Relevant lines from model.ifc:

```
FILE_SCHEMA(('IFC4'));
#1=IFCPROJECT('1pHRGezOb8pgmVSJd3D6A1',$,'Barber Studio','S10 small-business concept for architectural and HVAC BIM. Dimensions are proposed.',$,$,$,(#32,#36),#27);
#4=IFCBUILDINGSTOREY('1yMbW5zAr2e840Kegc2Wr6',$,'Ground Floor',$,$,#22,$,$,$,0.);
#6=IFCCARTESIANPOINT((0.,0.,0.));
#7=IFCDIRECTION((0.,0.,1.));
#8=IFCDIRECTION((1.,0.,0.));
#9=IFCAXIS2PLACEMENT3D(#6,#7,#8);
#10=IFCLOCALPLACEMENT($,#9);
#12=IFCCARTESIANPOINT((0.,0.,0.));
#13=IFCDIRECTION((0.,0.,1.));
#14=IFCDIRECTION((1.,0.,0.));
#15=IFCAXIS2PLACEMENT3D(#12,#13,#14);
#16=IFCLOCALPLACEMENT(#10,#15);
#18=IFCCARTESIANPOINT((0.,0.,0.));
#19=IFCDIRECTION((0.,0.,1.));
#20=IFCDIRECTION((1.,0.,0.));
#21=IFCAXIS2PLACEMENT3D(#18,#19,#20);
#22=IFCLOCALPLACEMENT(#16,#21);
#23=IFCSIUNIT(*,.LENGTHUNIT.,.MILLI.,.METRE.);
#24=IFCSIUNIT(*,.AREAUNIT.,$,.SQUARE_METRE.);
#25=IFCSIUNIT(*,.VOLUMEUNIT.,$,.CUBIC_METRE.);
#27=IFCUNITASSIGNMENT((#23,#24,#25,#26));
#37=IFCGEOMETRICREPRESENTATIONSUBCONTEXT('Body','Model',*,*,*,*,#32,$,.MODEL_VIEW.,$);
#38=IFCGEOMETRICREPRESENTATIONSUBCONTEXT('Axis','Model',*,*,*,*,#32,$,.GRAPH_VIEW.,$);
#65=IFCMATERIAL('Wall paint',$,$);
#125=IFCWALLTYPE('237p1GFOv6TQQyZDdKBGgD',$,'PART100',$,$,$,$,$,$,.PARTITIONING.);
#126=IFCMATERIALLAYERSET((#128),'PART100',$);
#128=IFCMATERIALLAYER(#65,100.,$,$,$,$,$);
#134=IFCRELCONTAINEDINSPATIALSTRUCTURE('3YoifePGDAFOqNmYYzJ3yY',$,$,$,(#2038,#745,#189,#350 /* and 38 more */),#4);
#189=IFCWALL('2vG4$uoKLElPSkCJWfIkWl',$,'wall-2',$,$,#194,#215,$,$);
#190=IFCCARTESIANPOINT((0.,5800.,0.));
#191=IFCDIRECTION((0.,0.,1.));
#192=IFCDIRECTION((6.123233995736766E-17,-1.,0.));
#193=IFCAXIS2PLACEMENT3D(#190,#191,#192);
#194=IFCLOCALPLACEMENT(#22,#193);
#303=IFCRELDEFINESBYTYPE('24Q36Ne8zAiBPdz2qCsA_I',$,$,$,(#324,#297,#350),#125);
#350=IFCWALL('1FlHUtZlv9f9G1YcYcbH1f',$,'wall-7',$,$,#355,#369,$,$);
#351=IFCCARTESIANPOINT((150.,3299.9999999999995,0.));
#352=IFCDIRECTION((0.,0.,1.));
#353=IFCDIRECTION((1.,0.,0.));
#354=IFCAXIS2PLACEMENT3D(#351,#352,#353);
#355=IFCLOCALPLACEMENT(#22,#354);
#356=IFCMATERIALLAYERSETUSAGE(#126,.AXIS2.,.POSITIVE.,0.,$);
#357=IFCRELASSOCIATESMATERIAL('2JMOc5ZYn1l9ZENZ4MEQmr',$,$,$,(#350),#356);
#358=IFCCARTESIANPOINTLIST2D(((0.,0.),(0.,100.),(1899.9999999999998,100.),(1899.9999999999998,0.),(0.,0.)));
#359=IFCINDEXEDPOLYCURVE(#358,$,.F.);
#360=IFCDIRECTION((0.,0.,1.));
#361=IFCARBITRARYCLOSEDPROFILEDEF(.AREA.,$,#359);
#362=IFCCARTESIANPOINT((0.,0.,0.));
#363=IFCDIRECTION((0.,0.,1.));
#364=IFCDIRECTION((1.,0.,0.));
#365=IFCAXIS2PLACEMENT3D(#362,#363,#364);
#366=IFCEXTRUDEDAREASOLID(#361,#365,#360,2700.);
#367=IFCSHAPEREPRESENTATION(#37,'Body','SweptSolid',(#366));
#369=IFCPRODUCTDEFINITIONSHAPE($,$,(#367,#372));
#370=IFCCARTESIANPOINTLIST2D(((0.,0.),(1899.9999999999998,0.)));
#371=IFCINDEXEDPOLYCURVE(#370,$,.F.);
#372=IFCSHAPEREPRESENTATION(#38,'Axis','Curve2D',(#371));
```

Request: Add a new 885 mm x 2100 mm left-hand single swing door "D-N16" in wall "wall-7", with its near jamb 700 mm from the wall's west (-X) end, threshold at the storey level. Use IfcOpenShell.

```python
import numpy as np
import ifcopenshell
import ifcopenshell.api.feature
import ifcopenshell.api.geometry
import ifcopenshell.api.root
import ifcopenshell.api.spatial
import ifcopenshell.geom
import ifcopenshell.util.element
import ifcopenshell.util.placement
import ifcopenshell.util.representation
import ifcopenshell.util.shape
import ifcopenshell.util.unit

model = ifcopenshell.open("model.ifc")
unit_scale = ifcopenshell.util.unit.calculate_unit_scale(model)
settings = ifcopenshell.geom.settings()


def volume(element):
    """Net volume in cubic metres, openings subtracted."""
    shape = ifcopenshell.geom.create_shape(settings, element)
    return ifcopenshell.util.shape.get_volume(shape.geometry)


wall = model.by_guid("1FlHUtZlv9f9G1YcYcbH1f")
storey = ifcopenshell.util.element.get_container(wall, ifc_class="IfcBuildingStorey")
context = ifcopenshell.util.representation.get_context(model, "Model", "Body", "MODEL_VIEW")
before = volume(wall)

width, height, from_end, sill = 0.885, 2.1, 0.7, 0.0  # metres

# The wall runs along its own X axis, and the end named is its -X end.
wall_shape = ifcopenshell.geom.create_shape(settings, wall)
x, y, z = ifcopenshell.util.shape.get_vertices(wall_shape.geometry).T
start = x.min() + from_end
face, thickness = float(y.min()), float(y.max() - y.min())
wall_matrix = ifcopenshell.util.placement.get_local_placement(wall.ObjectPlacement)
level = ifcopenshell.util.placement.get_local_placement(storey.ObjectPlacement)[2, 3]


def in_wall(x, y):
    """Placement at x, y metres in the wall's axes, at sill height."""
    matrix = wall_matrix.copy()
    matrix[:, 3] = wall_matrix @ np.array([x / unit_scale, y / unit_scale, 0.0, 1.0])
    matrix[2, 3] = level + sill / unit_scale
    return matrix


# Opening: a box that overshoots both wall faces by 50 mm.
opening = ifcopenshell.api.root.create_entity(model, ifc_class="IfcOpeningElement", predefined_type="OPENING")
box = ifcopenshell.api.geometry.add_wall_representation(
    model, context=context, length=width, height=height, thickness=thickness + 0.1
)
ifcopenshell.api.geometry.assign_representation(model, product=opening, representation=box)
ifcopenshell.api.geometry.edit_object_placement(model, product=opening, matrix=in_wall(start, face - 0.05), is_si=False)
ifcopenshell.api.feature.add_feature(model, feature=opening, element=wall)

door = ifcopenshell.api.root.create_entity(model, ifc_class="IfcDoor", name="D-N16", predefined_type="DOOR")
door.OverallWidth, door.OverallHeight = width / unit_scale, height / unit_scale
door.OperationType = "SINGLE_SWING_LEFT"
body = ifcopenshell.api.geometry.add_door_representation(
    model,
    context=context,
    overall_width=door.OverallWidth,
    overall_height=door.OverallHeight,
    operation_type="SINGLE_SWING_LEFT",
    lining_properties={"LiningDepth": thickness / unit_scale, "ThresholdDepth": thickness / unit_scale},
)
ifcopenshell.api.geometry.assign_representation(model, product=door, representation=body)
ifcopenshell.api.spatial.assign_container(model, products=[door], relating_structure=storey)
ifcopenshell.api.feature.add_filling(model, opening=opening, element=door)

# The lining spans the wall, so the door starts at the wall face.
ifcopenshell.api.geometry.edit_object_placement(model, product=door, matrix=in_wall(start, face), is_si=False)

after = volume(wall)

print(f"wall volume {before:.3f} -> {after:.3f} m3")

model.write("model-out.ifc")
```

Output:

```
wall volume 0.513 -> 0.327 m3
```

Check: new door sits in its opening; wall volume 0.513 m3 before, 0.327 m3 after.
